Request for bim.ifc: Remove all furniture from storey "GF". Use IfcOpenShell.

First a look at what the model holds.

```python
import ifcopenshell
import ifcopenshell.util.element

model = ifcopenshell.open("bim.ifc")
print(model.schema)
storey = next(s for s in model.by_type("IfcBuildingStorey") if s.Name == "GF")
furniture = [e for e in ifcopenshell.util.element.get_decomposition(storey) if e.is_a("IfcFurnishingElement")]
seen = {}
for e in furniture:
    element_type = ifcopenshell.util.element.get_type(e)
    name = element_type.Name if element_type not in (None, e) else None
    seen[name] = seen.get(name, 0) + 1
for name, count in sorted(seen.items(), key=str):
    print(count, "x", name)
```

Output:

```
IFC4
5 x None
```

```python
import ifcopenshell
import ifcopenshell.api.root
import ifcopenshell.util.element

model = ifcopenshell.open("bim.ifc")

storey = next(s for s in model.by_type("IfcBuildingStorey") if s.Name == "GF")
furniture = [e for e in ifcopenshell.util.element.get_decomposition(storey) if e.is_a("IfcFurnishingElement")]

for e in furniture:
    ifcopenshell.api.root.remove_product(model, product=e)
print(len(furniture), "removed")

model.write("bim_v2.ifc")
```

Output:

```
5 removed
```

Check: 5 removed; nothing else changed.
